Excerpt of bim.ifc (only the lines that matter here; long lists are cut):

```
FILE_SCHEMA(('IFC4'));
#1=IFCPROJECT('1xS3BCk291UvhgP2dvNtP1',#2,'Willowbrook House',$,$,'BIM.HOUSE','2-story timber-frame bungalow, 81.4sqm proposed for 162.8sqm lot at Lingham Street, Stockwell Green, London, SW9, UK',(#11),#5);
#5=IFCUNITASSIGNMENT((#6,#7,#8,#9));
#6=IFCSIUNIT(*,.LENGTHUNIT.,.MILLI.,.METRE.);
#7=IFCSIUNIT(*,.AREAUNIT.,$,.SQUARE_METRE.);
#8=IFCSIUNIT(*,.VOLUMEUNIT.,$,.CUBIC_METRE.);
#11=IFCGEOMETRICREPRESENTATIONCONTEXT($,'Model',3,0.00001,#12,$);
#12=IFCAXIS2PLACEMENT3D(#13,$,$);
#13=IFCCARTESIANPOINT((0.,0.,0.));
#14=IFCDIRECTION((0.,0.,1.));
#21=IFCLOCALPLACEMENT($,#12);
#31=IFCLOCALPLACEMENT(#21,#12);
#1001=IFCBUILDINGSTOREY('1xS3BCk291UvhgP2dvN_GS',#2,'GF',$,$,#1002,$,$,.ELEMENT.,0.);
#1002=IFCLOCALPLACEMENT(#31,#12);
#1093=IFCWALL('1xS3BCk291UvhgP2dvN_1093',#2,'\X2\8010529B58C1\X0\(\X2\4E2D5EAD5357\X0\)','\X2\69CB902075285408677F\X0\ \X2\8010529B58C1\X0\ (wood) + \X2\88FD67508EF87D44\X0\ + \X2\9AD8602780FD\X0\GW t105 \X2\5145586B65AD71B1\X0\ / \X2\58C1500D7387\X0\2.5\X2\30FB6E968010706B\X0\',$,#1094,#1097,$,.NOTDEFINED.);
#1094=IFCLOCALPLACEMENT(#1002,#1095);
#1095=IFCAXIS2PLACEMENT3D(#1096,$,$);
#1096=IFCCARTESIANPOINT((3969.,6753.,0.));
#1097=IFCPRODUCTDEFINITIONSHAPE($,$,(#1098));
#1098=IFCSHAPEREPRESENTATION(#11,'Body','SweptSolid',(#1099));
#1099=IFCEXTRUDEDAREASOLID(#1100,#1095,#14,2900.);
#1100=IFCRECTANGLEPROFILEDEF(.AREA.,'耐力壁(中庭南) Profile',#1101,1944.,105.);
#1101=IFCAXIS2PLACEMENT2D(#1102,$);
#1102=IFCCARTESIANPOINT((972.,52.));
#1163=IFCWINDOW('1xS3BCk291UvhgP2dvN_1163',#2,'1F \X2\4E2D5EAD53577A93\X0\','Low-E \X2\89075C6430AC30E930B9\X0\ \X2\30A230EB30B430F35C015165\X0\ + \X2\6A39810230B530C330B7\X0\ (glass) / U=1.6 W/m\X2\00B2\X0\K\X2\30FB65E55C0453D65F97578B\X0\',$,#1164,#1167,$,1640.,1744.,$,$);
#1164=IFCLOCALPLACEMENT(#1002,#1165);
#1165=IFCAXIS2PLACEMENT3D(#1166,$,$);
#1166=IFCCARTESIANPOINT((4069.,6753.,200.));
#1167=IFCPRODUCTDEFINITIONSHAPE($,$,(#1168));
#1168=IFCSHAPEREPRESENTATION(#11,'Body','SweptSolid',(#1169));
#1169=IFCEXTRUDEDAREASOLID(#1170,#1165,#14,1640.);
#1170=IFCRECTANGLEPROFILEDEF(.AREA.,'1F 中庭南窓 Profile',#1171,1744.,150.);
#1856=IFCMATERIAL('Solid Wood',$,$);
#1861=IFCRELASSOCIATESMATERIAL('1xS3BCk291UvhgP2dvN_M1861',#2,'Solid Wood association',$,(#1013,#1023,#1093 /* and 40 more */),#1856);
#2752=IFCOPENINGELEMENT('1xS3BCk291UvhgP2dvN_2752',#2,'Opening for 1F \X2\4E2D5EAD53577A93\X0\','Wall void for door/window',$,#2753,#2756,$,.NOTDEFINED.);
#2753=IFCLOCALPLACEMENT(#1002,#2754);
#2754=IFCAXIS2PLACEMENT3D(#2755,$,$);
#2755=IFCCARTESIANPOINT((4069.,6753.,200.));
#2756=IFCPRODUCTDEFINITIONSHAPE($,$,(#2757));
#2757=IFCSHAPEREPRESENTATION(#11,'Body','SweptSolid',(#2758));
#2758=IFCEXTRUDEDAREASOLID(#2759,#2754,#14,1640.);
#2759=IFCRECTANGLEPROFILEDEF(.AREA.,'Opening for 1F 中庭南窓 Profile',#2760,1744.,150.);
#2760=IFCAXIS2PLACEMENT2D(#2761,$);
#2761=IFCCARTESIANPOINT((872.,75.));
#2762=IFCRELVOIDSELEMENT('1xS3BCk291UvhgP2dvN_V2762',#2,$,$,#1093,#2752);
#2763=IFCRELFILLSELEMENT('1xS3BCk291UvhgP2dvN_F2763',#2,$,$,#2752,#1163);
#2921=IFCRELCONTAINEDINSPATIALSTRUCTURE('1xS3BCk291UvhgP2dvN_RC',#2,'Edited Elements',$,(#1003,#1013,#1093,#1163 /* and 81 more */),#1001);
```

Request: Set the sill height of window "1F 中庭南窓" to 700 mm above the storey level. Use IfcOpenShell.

```python
import numpy as np
import ifcopenshell
import ifcopenshell.api.geometry
import ifcopenshell.geom
import ifcopenshell.util.element
import ifcopenshell.util.placement
import ifcopenshell.util.shape
import ifcopenshell.util.unit

model = ifcopenshell.open("bim.ifc")
unit_scale = ifcopenshell.util.unit.calculate_unit_scale(model)

window = model.by_id(1163)
opening = window.FillsVoids[0].RelatingOpeningElement
storey = ifcopenshell.util.element.get_container(window, ifc_class="IfcBuildingStorey")
level = ifcopenshell.util.placement.get_local_placement(storey.ObjectPlacement)[2, 3]

# The opening's origin need not be at the sill, so measure its lowest point.
shape = ifcopenshell.geom.create_shape(ifcopenshell.geom.settings(), opening)
bottom = ifcopenshell.util.shape.get_shape_bottom_elevation(shape, shape.geometry) / unit_scale
dz = level + 700.0 - bottom

shift = np.array([0.0, 0.0, dz])
# The window is not placed relative to its opening, so move both.
for product in (opening, window):
    matrix = ifcopenshell.util.placement.get_local_placement(product.ObjectPlacement)
    matrix[:3, 3] += shift
    ifcopenshell.api.geometry.edit_object_placement(model, product=product, matrix=matrix, is_si=False)

print(f"moved by {dz * unit_scale:+.3f} m")

model.write("bim_updated.ifc")
```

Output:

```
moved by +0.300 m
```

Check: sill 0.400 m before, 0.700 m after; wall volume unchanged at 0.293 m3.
